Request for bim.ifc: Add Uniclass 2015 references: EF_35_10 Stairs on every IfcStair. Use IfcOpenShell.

First a look at what the model holds.

```python
import ifcopenshell

model = ifcopenshell.open("bim.ifc")
print(model.schema)
print("classifications:", [c.Name for c in model.by_type("IfcClassification")])
for ifc_class in ("IfcDoor", "IfcRoof", "IfcStair", "IfcWall", "IfcWindow"):
    print(ifc_class, len(model.by_type(ifc_class)))
```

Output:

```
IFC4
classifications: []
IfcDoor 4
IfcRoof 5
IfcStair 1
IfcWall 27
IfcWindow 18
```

```python
import ifcopenshell
import ifcopenshell.api.classification

model = ifcopenshell.open("bim.ifc")

system = ifcopenshell.api.classification.add_classification(model, classification="Uniclass 2015")

codes = {
    "IfcStair": ("EF_35_10", "Stairs"),
}
for ifc_class, (code, name) in codes.items():
    products = model.by_type(ifc_class)
    ifcopenshell.api.classification.add_reference(
        model, products=products, classification=system, identification=code, name=name
    )
    print(code, len(products))

model.write("bim_updated.ifc")
```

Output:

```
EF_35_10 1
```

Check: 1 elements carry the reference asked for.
